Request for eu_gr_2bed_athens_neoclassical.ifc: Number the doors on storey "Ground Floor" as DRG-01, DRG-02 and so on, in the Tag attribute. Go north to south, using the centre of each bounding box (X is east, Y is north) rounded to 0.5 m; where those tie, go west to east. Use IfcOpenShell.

First a look at what the model holds.

```python
import ifcopenshell
import ifcopenshell.util.element
import ifcopenshell.util.placement

model = ifcopenshell.open("eu_gr_2bed_athens_neoclassical.ifc")
print(model.schema)
storey = next(s for s in model.by_type("IfcBuildingStorey") if s.Name == "Ground Floor")
doors = [e for e in ifcopenshell.util.element.get_decomposition(storey) if e.is_a("IfcDoor")]
for e in sorted(doors, key=lambda e: e.id()):
    origin = ifcopenshell.util.placement.get_local_placement(e.ObjectPlacement)[:3, 3]
    print(e.id(), e.Tag, e.Name, origin.round(2) + 0.0, sep=" | ")
```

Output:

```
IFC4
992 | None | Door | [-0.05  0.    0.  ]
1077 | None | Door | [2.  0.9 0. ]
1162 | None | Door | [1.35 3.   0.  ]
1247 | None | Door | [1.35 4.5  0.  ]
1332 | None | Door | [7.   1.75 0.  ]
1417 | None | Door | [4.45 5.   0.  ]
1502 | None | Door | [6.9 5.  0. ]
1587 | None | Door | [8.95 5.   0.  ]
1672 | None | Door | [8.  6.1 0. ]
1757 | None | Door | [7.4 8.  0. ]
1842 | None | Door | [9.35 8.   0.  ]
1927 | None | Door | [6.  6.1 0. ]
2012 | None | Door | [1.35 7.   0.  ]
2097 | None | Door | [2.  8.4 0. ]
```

```python
import ifcopenshell
import ifcopenshell.geom
import ifcopenshell.util.element
import ifcopenshell.util.shape

model = ifcopenshell.open("eu_gr_2bed_athens_neoclassical.ifc")
settings = ifcopenshell.geom.settings()
settings.set("use-world-coords", True)


def centre(element):
    shape = ifcopenshell.geom.create_shape(settings, element)
    return ifcopenshell.util.shape.get_bbox_centroid(shape.geometry)


storey = next(s for s in model.by_type("IfcBuildingStorey") if s.Name == "Ground Floor")
doors = [e for e in ifcopenshell.util.element.get_decomposition(storey) if e.is_a("IfcDoor")]

# Insertion points can sit at a corner or the storey origin, so sort by the geometry (in metres).
centres = {e: centre(e) for e in doors}
doors.sort(key=lambda e: (-round(centres[e][1] / 0.5), centres[e][0]))

for i, e in enumerate(doors, start=1):
    number = f"DRG-{i:02d}"
    e.Tag = number
    print(e.id(), number)

model.write("eu_gr_2bed_athens_neoclassical_rev.ifc")
```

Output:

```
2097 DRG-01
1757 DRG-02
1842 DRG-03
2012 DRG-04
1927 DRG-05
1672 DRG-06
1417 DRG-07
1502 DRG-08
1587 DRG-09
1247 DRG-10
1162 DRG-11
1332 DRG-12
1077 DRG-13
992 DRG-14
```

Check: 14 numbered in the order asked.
